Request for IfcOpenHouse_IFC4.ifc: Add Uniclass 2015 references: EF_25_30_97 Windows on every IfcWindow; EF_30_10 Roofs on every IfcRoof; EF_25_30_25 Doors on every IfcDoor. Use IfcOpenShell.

First a look at what the model holds.

```python
import ifcopenshell

model = ifcopenshell.open("IfcOpenHouse_IFC4.ifc")
print(model.schema)
print("classifications:", [c.Name for c in model.by_type("IfcClassification")])
for ifc_class in ("IfcDoor", "IfcRoof", "IfcStair", "IfcWall", "IfcWindow"):
    print(ifc_class, len(model.by_type(ifc_class)))
```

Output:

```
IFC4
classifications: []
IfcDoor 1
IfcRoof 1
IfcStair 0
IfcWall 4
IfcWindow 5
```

```python
import ifcopenshell
import ifcopenshell.api.classification

model = ifcopenshell.open("IfcOpenHouse_IFC4.ifc")

system = ifcopenshell.api.classification.add_classification(model, classification="Uniclass 2015")

codes = {
    "IfcWindow": ("EF_25_30_97", "Windows"),
    "IfcRoof": ("EF_30_10", "Roofs"),
    "IfcDoor": ("EF_25_30_25", "Doors"),
}
for ifc_class, (code, name) in codes.items():
    products = model.by_type(ifc_class)
    ifcopenshell.api.classification.add_reference(
        model, products=products, classification=system, identification=code, name=name
    )
    print(code, len(products))

model.write("IfcOpenHouse_IFC4_rev.ifc")
```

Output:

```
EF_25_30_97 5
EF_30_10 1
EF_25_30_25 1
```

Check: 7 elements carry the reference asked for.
